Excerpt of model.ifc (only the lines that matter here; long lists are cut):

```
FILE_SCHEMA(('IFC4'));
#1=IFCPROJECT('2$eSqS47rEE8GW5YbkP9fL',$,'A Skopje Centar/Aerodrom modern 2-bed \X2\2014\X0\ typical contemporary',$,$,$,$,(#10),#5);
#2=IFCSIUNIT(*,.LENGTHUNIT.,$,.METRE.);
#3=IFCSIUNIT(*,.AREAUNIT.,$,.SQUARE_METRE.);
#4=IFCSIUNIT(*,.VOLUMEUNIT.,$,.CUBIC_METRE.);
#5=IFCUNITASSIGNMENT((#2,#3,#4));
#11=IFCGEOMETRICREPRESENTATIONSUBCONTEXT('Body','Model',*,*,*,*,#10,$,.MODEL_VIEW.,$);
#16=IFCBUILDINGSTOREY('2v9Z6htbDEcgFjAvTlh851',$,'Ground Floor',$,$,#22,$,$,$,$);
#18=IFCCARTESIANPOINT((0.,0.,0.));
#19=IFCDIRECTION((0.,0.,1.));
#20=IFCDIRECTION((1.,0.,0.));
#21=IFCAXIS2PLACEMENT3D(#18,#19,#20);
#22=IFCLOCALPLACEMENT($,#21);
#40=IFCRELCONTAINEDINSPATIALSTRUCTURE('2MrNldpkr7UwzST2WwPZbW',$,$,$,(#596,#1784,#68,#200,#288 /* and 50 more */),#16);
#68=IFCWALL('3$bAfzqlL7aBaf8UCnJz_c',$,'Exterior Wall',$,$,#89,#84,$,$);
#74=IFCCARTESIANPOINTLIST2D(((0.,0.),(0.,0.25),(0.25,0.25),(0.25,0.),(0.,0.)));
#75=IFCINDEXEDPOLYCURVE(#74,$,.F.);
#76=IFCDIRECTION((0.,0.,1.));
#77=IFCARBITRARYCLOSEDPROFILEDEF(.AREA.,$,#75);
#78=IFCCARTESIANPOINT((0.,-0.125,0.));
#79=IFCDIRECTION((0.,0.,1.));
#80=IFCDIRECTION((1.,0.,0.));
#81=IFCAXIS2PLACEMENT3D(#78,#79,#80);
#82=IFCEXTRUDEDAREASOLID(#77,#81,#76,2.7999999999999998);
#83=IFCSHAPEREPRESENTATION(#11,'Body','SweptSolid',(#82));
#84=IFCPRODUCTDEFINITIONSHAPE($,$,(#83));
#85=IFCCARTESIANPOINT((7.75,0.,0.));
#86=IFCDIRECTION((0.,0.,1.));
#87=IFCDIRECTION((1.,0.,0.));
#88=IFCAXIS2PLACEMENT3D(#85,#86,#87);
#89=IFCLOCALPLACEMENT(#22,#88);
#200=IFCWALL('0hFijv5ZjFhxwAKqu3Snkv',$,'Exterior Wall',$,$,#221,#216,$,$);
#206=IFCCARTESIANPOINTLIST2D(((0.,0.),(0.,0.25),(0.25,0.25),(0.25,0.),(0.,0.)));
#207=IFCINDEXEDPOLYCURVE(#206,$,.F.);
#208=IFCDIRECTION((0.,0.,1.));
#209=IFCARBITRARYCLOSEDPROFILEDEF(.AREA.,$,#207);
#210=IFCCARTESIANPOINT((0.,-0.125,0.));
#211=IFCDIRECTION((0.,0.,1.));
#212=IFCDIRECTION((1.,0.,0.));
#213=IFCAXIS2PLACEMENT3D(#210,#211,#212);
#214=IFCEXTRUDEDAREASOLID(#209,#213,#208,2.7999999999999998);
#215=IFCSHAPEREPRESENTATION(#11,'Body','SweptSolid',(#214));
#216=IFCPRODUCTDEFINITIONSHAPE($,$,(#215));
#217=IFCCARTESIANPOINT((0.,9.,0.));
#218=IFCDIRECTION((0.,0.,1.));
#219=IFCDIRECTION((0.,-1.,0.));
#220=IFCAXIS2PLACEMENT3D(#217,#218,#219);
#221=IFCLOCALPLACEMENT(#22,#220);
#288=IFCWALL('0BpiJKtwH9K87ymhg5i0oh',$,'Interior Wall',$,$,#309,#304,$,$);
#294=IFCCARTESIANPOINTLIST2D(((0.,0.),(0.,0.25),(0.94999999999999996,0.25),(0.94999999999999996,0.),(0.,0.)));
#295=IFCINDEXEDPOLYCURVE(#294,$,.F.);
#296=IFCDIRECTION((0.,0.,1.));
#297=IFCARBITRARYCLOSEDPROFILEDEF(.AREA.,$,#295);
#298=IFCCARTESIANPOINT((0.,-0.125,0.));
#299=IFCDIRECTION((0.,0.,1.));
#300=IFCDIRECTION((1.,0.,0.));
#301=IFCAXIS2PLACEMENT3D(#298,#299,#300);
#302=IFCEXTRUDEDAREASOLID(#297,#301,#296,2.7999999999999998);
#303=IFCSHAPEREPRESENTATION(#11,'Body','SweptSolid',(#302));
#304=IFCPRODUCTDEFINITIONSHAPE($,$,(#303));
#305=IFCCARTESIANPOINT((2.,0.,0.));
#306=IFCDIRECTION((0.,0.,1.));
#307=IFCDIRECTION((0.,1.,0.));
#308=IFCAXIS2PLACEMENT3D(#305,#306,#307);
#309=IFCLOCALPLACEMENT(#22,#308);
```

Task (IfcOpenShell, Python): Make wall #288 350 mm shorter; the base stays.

```python
import ifcopenshell
import ifcopenshell.geom
import ifcopenshell.util.representation
import ifcopenshell.util.shape

model = ifcopenshell.open("model.ifc")
settings = ifcopenshell.geom.settings()


def volume(element):
    """Net volume in cubic metres, openings subtracted."""
    shape = ifcopenshell.geom.create_shape(settings, element)
    return ifcopenshell.util.shape.get_volume(shape.geometry)


wall = model.by_guid("0BpiJKtwH9K87ymhg5i0oh")
before = volume(wall)

body = ifcopenshell.util.representation.get_representation(wall, "Model", "Body")
solid = body.Items[0]
old_height = solid.Depth
solid.Depth -= 0.35
after = volume(wall)

print(f"height {old_height:g} -> {solid.Depth:g}, volume {before:.3f} -> {after:.3f} m3")

model.write("model_edited.ifc")
```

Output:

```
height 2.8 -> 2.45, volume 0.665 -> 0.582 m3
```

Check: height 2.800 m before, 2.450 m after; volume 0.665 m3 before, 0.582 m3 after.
